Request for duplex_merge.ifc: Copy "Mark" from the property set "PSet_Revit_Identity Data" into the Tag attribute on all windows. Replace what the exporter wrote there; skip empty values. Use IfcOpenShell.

First a look at what the model holds.

```python
import ifcopenshell
import ifcopenshell.util.element

model = ifcopenshell.open("duplex_merge.ifc")
print(model.schema)
windows = model.by_type("IfcWindow")
print(len(windows), "windows")
for e in windows[:8]:
    source = ifcopenshell.util.element.get_pset(e, "PSet_Revit_Identity Data", "Mark")
    target = e.Tag
    print(e.id(), repr(source), repr(target), sep=" | ")
```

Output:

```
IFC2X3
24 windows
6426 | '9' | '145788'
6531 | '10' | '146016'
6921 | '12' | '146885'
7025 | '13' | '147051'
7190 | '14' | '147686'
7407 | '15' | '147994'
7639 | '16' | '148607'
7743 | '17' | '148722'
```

```python
import ifcopenshell
import ifcopenshell.util.element

model = ifcopenshell.open("duplex_merge.ifc")

count = 0
for e in model.by_type("IfcWindow"):
    value = ifcopenshell.util.element.get_pset(e, "PSet_Revit_Identity Data", "Mark")
    current = e.Tag
    if not value or not value.strip() or current == value:
        continue
    e.Tag = value
    count += 1

print(count, "windows updated")

model.write("duplex_merge-out.ifc")
```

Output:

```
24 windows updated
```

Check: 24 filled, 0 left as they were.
